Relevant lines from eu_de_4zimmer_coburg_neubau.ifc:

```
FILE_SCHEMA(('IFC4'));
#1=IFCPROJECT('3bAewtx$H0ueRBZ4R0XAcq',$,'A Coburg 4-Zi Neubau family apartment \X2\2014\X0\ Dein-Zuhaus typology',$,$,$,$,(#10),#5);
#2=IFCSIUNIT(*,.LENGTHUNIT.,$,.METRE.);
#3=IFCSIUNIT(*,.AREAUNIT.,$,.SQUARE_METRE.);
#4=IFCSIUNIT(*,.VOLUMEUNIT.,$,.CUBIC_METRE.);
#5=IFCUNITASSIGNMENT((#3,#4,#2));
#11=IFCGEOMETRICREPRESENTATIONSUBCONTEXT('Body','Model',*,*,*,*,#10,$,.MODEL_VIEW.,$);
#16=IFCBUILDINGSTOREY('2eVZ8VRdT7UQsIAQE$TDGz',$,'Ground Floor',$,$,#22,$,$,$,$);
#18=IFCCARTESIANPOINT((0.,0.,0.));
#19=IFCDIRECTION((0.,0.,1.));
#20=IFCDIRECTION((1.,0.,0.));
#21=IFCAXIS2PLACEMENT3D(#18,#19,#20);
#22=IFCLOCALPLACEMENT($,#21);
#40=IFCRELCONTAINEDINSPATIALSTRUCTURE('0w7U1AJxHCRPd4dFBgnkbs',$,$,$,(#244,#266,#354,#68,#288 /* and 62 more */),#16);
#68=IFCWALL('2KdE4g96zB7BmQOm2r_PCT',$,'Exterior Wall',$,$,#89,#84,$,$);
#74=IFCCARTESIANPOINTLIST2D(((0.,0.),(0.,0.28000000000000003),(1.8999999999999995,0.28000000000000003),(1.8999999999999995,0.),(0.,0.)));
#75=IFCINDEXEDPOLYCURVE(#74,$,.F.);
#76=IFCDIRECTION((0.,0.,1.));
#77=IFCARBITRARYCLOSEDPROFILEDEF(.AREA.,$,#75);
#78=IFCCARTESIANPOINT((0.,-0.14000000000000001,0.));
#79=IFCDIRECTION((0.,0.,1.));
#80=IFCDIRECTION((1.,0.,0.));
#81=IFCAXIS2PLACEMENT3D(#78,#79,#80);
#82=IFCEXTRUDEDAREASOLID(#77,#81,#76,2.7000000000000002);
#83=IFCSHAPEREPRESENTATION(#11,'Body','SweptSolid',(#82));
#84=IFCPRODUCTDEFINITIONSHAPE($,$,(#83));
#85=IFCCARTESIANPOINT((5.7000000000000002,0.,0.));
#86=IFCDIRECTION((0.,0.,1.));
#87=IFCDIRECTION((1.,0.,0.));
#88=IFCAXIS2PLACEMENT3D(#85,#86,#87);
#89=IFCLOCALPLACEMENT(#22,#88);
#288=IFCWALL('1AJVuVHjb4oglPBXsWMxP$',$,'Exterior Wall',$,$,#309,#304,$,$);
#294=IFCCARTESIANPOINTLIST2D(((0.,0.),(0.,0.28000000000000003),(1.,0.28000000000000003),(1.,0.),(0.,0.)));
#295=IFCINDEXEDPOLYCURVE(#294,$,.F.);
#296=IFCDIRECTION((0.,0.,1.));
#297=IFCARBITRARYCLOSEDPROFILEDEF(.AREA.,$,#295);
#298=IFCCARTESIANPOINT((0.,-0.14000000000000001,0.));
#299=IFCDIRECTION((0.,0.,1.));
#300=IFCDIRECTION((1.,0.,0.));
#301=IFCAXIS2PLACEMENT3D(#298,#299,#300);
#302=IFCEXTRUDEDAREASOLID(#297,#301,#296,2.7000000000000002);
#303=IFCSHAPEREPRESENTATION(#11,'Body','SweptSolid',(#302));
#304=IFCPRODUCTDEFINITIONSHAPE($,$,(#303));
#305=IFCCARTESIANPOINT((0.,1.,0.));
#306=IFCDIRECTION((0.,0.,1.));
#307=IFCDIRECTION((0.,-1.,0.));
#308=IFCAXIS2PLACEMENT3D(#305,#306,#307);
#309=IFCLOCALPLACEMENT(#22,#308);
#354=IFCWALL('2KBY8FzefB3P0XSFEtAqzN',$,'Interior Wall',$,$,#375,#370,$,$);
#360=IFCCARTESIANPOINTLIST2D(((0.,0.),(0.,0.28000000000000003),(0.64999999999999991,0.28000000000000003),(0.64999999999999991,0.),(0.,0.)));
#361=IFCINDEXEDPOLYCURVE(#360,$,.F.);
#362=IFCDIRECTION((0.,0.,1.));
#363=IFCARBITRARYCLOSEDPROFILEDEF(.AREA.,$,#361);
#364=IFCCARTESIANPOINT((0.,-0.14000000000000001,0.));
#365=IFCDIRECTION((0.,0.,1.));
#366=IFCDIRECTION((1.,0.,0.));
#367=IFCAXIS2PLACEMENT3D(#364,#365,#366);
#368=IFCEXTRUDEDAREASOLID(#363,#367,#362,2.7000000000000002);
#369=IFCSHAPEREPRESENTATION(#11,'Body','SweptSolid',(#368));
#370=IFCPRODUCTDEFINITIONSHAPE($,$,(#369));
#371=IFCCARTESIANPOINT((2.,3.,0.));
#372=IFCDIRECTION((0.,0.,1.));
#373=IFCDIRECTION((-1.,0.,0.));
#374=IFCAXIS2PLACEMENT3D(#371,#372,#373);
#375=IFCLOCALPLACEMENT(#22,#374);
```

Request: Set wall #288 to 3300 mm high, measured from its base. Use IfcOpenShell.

```python
import ifcopenshell
import ifcopenshell.geom
import ifcopenshell.util.representation
import ifcopenshell.util.shape

model = ifcopenshell.open("eu_de_4zimmer_coburg_neubau.ifc")
settings = ifcopenshell.geom.settings()


def volume(element):
    """Net volume in cubic metres, openings subtracted."""
    shape = ifcopenshell.geom.create_shape(settings, element)
    return ifcopenshell.util.shape.get_volume(shape.geometry)


wall = model.by_id(288)
before = volume(wall)

body = ifcopenshell.util.representation.get_representation(wall, "Model", "Body")
solid = body.Items[0]
old_height = solid.Depth
solid.Depth = 3.3
after = volume(wall)

print(f"height {old_height:g} -> {solid.Depth:g}, volume {before:.3f} -> {after:.3f} m3")

model.write("eu_de_4zimmer_coburg_neubau_v2.ifc")
```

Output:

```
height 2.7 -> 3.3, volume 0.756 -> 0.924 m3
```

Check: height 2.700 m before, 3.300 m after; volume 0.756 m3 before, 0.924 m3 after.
